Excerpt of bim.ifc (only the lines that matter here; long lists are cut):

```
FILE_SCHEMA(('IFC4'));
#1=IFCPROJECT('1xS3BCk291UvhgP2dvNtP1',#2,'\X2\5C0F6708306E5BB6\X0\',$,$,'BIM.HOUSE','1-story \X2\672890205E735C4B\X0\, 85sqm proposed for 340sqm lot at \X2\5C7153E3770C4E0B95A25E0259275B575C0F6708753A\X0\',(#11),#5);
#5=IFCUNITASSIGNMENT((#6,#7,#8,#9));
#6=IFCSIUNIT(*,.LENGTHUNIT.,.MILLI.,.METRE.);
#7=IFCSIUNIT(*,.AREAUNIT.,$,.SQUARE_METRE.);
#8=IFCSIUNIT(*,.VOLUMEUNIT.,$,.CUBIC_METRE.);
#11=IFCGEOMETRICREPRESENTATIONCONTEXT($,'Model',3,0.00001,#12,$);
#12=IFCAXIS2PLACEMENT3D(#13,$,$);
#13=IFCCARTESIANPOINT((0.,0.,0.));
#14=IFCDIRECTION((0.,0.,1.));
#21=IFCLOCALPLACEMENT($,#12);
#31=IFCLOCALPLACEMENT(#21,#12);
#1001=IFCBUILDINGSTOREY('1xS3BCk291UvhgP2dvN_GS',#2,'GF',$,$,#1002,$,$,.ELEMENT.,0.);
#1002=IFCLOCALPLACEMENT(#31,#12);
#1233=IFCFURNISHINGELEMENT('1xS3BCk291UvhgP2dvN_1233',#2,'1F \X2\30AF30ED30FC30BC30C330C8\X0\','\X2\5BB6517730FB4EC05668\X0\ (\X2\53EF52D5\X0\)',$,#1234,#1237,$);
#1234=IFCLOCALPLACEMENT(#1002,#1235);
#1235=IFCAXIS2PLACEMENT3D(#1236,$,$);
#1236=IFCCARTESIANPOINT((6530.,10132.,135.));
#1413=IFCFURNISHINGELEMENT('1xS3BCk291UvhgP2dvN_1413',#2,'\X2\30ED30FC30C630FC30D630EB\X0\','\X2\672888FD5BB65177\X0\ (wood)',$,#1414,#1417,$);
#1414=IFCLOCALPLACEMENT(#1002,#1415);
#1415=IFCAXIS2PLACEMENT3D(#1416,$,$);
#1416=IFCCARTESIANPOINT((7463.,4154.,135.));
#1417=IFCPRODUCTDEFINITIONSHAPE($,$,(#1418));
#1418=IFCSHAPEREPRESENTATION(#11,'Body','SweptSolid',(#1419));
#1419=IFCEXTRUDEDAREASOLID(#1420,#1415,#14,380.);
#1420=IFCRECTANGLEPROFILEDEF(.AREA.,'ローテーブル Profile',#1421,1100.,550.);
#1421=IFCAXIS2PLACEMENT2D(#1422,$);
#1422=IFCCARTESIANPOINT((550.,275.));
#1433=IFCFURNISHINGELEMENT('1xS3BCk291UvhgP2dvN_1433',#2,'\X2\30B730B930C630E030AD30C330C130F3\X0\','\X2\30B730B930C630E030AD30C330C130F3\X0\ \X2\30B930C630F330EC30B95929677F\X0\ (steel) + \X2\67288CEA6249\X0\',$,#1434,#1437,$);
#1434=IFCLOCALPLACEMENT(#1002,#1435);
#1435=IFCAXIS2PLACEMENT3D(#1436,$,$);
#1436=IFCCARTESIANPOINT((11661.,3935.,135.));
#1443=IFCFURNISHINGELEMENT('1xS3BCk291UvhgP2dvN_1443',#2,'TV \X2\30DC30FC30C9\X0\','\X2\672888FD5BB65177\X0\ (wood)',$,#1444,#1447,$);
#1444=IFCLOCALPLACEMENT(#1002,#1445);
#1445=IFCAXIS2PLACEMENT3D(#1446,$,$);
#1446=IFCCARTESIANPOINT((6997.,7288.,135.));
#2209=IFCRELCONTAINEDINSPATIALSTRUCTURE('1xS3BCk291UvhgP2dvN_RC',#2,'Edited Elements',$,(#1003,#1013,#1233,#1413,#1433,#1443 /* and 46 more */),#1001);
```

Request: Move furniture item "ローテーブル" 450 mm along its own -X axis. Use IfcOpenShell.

```python
import ifcopenshell
import ifcopenshell.api.geometry
import ifcopenshell.util.placement

model = ifcopenshell.open("bim.ifc")

item = model.by_id(1413)
matrix = ifcopenshell.util.placement.get_local_placement(item.ObjectPlacement)
matrix[:3, 3] -= matrix[:3, 0] * 450.0
ifcopenshell.api.geometry.edit_object_placement(model, product=item, matrix=matrix, is_si=False)

print(ifcopenshell.util.placement.get_local_placement(item.ObjectPlacement).round(3) + 0.0)

model.write("bim-out.ifc")
```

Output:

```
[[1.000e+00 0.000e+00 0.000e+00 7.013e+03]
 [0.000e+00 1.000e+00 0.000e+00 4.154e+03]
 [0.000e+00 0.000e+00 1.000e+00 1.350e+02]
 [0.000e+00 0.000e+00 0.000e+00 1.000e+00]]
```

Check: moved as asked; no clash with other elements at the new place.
